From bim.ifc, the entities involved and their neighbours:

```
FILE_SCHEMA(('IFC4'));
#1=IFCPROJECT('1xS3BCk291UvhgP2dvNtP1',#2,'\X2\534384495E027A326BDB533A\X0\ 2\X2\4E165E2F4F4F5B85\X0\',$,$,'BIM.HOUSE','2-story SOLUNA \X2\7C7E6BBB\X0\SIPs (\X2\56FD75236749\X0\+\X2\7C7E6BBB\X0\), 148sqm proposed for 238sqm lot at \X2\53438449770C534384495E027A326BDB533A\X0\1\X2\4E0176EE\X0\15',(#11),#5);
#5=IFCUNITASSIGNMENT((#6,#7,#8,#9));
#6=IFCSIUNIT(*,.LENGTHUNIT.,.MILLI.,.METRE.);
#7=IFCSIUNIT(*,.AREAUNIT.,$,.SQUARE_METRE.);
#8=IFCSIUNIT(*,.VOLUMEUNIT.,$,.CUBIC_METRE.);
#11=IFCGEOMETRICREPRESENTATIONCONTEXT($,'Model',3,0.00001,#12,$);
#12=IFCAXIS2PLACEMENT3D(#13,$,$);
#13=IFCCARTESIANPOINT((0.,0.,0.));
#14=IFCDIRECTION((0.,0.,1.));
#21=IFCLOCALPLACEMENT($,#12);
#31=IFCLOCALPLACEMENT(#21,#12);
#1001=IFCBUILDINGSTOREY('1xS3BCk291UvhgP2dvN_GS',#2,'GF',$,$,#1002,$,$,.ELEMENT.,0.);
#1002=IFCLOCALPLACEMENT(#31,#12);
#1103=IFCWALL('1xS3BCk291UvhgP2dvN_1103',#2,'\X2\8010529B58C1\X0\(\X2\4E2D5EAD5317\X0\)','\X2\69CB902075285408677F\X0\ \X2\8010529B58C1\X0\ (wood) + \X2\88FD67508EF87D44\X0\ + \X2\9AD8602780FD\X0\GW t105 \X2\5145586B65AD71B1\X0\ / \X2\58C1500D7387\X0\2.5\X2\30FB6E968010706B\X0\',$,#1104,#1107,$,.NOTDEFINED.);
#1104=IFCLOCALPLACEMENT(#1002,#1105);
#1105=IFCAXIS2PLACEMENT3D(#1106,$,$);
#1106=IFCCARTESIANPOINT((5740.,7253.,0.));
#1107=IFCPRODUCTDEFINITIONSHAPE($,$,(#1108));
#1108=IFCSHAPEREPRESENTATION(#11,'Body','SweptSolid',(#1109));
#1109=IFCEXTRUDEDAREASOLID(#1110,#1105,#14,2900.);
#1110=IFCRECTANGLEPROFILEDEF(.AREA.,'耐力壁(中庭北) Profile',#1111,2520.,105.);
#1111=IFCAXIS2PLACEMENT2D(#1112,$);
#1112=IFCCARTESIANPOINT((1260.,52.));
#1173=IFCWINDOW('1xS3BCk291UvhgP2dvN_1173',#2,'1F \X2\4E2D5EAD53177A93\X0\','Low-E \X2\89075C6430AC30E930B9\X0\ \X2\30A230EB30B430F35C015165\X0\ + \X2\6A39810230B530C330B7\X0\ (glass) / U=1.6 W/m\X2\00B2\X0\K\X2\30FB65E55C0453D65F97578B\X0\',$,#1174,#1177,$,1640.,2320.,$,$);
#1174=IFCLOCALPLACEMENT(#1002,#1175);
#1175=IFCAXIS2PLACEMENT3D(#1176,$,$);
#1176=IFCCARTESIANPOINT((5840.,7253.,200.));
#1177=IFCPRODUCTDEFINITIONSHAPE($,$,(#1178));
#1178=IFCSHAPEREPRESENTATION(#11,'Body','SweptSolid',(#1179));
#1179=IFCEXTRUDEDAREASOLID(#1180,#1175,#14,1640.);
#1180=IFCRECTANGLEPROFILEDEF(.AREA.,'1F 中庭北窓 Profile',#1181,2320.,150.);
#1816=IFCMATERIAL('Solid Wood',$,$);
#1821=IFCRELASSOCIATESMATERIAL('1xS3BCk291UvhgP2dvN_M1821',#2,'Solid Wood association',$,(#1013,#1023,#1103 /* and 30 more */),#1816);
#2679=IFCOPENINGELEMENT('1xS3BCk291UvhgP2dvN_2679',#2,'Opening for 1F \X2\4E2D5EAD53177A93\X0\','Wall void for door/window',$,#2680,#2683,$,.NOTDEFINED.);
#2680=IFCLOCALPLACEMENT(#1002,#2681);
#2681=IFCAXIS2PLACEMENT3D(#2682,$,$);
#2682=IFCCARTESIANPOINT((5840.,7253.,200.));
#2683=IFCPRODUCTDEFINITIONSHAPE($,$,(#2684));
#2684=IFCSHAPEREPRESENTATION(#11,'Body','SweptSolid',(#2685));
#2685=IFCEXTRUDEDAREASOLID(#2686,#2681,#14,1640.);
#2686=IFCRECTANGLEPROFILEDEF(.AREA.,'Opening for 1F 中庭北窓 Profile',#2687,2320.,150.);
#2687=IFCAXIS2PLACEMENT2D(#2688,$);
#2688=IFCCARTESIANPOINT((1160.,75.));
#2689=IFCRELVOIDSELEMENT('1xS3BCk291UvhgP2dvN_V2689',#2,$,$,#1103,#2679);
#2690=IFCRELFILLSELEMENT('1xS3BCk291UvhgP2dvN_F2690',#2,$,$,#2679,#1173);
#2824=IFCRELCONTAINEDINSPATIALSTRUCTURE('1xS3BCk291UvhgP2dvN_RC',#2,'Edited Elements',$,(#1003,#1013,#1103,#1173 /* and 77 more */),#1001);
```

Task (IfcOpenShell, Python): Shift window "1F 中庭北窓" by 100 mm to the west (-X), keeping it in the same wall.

```python
import ifcopenshell
import ifcopenshell.api.geometry
import ifcopenshell.util.placement
import ifcopenshell.util.unit

model = ifcopenshell.open("bim.ifc")
unit_scale = ifcopenshell.util.unit.calculate_unit_scale(model)

window = model.by_guid("1xS3BCk291UvhgP2dvN_1173")
opening = window.FillsVoids[0].RelatingOpeningElement
wall = opening.VoidsElements[0].RelatingBuildingElement

wall_matrix = ifcopenshell.util.placement.get_local_placement(wall.ObjectPlacement)
shift = wall_matrix[:3, 0] * -0.1 / unit_scale
before = ifcopenshell.util.placement.get_local_placement(window.ObjectPlacement)[:3, 3].copy()

# The window is not placed relative to its opening, so move both.
for product in (opening, window):
    matrix = ifcopenshell.util.placement.get_local_placement(product.ObjectPlacement)
    matrix[:3, 3] += shift
    ifcopenshell.api.geometry.edit_object_placement(model, product=product, matrix=matrix, is_si=False)

after = ifcopenshell.util.placement.get_local_placement(window.ObjectPlacement)[:3, 3]
print("window moved by", (after - before).round(3) + 0.0)

model.write("bim-out.ifc")
```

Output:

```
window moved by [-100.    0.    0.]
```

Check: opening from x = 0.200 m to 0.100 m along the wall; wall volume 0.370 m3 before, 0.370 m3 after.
